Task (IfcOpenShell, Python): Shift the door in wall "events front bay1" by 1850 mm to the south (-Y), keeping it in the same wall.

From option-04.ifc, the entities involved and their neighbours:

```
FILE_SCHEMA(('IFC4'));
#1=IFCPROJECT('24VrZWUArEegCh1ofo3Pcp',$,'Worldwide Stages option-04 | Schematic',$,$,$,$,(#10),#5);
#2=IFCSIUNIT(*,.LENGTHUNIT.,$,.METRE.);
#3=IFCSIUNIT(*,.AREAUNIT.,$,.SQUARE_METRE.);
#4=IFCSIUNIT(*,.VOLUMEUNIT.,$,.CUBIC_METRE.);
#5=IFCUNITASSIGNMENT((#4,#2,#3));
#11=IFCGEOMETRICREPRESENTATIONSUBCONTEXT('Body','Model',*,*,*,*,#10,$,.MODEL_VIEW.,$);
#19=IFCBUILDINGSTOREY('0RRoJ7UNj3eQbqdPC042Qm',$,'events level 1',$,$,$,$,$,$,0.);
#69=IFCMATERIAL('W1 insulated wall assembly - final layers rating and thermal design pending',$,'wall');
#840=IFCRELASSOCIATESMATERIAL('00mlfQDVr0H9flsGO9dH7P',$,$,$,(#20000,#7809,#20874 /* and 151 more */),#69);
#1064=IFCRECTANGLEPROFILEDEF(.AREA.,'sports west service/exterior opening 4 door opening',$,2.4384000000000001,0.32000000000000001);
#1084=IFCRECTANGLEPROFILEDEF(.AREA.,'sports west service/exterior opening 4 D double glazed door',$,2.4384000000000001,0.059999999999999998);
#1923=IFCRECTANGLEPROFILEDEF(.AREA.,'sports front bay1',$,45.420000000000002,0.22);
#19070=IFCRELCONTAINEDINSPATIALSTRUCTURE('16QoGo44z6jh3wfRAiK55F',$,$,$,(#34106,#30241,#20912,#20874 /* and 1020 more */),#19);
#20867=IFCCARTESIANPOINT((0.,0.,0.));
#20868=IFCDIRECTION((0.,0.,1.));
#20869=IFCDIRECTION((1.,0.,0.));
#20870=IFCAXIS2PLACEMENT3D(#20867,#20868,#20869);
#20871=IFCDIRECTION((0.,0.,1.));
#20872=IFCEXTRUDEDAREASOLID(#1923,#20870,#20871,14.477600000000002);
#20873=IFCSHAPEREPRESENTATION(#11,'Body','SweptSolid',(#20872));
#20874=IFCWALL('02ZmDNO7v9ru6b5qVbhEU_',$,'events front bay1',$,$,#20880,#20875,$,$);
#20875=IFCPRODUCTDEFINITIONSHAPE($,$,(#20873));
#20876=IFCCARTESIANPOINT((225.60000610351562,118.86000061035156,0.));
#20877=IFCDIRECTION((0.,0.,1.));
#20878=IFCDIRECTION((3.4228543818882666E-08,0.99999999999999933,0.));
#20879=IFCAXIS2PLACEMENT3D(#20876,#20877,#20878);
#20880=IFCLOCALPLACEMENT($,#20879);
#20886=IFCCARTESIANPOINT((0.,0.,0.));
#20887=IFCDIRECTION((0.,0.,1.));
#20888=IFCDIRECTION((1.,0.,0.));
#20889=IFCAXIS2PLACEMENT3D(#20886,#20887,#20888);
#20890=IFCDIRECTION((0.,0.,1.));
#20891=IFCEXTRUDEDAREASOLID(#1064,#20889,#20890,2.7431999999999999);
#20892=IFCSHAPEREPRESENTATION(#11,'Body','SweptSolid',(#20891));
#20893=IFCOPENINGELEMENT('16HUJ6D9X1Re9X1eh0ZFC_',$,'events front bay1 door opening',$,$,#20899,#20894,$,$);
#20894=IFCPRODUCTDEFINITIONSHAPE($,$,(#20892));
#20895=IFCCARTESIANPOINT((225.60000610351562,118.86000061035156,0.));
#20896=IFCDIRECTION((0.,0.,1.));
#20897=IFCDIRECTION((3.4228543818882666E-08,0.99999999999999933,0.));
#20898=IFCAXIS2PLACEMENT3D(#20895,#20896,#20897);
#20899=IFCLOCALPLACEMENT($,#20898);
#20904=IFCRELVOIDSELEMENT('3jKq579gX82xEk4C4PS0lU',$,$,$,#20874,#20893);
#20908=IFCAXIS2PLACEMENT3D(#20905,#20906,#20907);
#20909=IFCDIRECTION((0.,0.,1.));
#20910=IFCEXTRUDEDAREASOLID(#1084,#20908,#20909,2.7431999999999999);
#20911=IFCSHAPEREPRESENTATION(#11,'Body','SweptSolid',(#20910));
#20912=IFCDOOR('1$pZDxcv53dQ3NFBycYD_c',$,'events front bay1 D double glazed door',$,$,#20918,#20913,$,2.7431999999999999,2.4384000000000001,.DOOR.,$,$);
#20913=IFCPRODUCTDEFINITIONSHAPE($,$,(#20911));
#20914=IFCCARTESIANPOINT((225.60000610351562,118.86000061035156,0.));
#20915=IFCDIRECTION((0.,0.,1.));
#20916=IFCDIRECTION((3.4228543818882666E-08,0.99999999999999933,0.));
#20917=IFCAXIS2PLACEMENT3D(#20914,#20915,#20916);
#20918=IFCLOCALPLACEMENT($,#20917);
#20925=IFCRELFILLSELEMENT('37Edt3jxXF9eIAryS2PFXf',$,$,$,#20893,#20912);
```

```python
import ifcopenshell
import ifcopenshell.api.geometry
import ifcopenshell.util.placement
import ifcopenshell.util.unit

model = ifcopenshell.open("option-04.ifc")
unit_scale = ifcopenshell.util.unit.calculate_unit_scale(model)

door = model.by_id(20912)
opening = door.FillsVoids[0].RelatingOpeningElement
wall = opening.VoidsElements[0].RelatingBuildingElement

wall_matrix = ifcopenshell.util.placement.get_local_placement(wall.ObjectPlacement)
shift = wall_matrix[:3, 0] * -1.85 / unit_scale
before = ifcopenshell.util.placement.get_local_placement(door.ObjectPlacement)[:3, 3].copy()

# The door is not placed relative to its opening, so move both.
for product in (opening, door):
    matrix = ifcopenshell.util.placement.get_local_placement(product.ObjectPlacement)
    matrix[:3, 3] += shift
    ifcopenshell.api.geometry.edit_object_placement(model, product=product, matrix=matrix, is_si=False)

after = ifcopenshell.util.placement.get_local_placement(door.ObjectPlacement)[:3, 3]
print("door moved by", (after - before).round(3) + 0.0)

model.write("option-04-out.ifc")
```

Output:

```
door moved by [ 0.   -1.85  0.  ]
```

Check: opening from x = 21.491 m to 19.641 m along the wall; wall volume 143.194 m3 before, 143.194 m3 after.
